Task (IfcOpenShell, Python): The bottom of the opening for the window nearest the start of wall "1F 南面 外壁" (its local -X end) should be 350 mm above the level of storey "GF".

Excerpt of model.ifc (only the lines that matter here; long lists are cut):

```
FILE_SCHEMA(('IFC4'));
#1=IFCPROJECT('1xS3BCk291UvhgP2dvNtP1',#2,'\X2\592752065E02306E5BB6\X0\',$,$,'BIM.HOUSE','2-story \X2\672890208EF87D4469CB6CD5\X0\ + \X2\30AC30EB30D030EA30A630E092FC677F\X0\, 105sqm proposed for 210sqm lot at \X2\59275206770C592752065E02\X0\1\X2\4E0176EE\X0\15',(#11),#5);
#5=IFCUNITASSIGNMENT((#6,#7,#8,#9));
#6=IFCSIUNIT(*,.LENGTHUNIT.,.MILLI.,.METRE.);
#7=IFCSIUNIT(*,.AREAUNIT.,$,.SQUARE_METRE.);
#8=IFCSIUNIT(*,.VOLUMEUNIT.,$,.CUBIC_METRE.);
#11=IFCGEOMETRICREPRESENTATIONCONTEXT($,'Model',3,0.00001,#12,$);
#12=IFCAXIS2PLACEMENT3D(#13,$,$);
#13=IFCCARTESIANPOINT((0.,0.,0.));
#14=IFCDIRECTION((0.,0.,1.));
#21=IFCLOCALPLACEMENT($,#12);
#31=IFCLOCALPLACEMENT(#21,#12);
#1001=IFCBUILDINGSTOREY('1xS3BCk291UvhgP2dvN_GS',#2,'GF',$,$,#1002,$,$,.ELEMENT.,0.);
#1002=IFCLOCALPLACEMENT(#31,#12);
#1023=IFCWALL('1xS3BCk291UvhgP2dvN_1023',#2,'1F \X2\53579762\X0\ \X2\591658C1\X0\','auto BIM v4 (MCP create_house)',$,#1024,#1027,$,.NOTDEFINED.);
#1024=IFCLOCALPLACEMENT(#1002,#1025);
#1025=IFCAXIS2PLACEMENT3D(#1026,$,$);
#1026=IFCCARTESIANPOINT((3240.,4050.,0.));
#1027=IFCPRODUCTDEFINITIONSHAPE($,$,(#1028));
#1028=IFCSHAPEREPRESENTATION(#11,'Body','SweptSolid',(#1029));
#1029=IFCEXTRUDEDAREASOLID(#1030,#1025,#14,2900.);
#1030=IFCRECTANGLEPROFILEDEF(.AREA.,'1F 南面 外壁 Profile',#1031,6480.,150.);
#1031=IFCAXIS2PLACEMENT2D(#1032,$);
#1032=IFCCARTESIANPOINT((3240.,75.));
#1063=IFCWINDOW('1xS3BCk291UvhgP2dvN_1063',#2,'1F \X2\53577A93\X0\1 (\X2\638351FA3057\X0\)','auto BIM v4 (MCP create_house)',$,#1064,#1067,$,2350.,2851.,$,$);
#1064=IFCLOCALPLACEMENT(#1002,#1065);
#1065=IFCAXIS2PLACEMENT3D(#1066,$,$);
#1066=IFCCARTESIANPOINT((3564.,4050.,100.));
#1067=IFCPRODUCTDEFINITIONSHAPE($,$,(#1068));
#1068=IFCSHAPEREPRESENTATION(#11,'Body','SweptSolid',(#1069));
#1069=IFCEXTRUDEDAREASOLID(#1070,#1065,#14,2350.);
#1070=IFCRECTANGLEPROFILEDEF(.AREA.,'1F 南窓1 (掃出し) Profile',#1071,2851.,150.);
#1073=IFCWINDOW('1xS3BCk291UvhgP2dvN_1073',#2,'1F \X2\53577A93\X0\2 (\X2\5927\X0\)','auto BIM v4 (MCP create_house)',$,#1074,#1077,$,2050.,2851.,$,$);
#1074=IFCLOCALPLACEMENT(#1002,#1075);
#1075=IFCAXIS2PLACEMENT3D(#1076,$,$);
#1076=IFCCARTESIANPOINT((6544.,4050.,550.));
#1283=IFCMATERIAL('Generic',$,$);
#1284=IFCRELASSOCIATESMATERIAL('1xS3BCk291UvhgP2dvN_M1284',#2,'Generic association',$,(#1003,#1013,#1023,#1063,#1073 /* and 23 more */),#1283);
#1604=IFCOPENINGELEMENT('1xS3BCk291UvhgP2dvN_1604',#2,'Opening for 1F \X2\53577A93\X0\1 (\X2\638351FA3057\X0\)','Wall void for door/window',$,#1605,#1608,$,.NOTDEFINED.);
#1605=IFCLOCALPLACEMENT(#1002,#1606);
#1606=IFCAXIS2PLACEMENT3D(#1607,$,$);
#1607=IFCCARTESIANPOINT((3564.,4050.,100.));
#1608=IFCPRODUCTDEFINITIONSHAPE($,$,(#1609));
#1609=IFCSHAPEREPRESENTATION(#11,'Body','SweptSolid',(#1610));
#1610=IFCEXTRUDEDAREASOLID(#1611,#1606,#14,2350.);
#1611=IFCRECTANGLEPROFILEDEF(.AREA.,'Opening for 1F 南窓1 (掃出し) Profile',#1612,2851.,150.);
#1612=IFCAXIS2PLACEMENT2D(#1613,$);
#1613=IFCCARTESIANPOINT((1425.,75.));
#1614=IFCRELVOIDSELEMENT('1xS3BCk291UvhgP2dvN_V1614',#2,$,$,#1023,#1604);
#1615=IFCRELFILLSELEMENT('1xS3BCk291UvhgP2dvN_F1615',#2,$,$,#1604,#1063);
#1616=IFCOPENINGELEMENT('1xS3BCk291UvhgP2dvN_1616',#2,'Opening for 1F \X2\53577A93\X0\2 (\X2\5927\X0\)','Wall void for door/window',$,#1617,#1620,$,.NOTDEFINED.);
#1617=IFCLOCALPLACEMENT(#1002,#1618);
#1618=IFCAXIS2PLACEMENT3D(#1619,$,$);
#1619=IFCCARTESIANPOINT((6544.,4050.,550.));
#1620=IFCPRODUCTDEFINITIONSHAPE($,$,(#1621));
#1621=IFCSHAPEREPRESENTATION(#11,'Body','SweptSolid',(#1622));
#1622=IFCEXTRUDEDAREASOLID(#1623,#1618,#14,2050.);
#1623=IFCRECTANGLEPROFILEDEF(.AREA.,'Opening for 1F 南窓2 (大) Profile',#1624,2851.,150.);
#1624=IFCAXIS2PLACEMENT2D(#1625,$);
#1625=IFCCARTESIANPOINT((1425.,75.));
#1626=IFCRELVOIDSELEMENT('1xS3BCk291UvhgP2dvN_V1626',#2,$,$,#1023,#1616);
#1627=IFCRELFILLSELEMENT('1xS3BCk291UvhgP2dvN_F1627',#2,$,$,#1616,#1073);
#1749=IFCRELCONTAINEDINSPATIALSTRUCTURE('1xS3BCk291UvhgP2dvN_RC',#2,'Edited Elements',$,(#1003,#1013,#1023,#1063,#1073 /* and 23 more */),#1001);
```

```python
import numpy as np
import ifcopenshell
import ifcopenshell.api.geometry
import ifcopenshell.geom
import ifcopenshell.util.element
import ifcopenshell.util.placement
import ifcopenshell.util.shape
import ifcopenshell.util.unit

model = ifcopenshell.open("model.ifc")
unit_scale = ifcopenshell.util.unit.calculate_unit_scale(model)

window = model.by_guid("1xS3BCk291UvhgP2dvN_1063")
opening = window.FillsVoids[0].RelatingOpeningElement
storey = ifcopenshell.util.element.get_container(window, ifc_class="IfcBuildingStorey")
level = ifcopenshell.util.placement.get_local_placement(storey.ObjectPlacement)[2, 3]

# The opening's origin need not be at the sill, so measure its lowest point.
shape = ifcopenshell.geom.create_shape(ifcopenshell.geom.settings(), opening)
bottom = ifcopenshell.util.shape.get_shape_bottom_elevation(shape, shape.geometry) / unit_scale
dz = level + 0.35 / unit_scale - bottom

shift = np.array([0.0, 0.0, dz])
# The window is not placed relative to its opening, so move both.
for product in (opening, window):
    matrix = ifcopenshell.util.placement.get_local_placement(product.ObjectPlacement)
    matrix[:3, 3] += shift
    ifcopenshell.api.geometry.edit_object_placement(model, product=product, matrix=matrix, is_si=False)

print(f"moved by {dz * unit_scale:+.3f} m")

model.write("model_rev.ifc")
```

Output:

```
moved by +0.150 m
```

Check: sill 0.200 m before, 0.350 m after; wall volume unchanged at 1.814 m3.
